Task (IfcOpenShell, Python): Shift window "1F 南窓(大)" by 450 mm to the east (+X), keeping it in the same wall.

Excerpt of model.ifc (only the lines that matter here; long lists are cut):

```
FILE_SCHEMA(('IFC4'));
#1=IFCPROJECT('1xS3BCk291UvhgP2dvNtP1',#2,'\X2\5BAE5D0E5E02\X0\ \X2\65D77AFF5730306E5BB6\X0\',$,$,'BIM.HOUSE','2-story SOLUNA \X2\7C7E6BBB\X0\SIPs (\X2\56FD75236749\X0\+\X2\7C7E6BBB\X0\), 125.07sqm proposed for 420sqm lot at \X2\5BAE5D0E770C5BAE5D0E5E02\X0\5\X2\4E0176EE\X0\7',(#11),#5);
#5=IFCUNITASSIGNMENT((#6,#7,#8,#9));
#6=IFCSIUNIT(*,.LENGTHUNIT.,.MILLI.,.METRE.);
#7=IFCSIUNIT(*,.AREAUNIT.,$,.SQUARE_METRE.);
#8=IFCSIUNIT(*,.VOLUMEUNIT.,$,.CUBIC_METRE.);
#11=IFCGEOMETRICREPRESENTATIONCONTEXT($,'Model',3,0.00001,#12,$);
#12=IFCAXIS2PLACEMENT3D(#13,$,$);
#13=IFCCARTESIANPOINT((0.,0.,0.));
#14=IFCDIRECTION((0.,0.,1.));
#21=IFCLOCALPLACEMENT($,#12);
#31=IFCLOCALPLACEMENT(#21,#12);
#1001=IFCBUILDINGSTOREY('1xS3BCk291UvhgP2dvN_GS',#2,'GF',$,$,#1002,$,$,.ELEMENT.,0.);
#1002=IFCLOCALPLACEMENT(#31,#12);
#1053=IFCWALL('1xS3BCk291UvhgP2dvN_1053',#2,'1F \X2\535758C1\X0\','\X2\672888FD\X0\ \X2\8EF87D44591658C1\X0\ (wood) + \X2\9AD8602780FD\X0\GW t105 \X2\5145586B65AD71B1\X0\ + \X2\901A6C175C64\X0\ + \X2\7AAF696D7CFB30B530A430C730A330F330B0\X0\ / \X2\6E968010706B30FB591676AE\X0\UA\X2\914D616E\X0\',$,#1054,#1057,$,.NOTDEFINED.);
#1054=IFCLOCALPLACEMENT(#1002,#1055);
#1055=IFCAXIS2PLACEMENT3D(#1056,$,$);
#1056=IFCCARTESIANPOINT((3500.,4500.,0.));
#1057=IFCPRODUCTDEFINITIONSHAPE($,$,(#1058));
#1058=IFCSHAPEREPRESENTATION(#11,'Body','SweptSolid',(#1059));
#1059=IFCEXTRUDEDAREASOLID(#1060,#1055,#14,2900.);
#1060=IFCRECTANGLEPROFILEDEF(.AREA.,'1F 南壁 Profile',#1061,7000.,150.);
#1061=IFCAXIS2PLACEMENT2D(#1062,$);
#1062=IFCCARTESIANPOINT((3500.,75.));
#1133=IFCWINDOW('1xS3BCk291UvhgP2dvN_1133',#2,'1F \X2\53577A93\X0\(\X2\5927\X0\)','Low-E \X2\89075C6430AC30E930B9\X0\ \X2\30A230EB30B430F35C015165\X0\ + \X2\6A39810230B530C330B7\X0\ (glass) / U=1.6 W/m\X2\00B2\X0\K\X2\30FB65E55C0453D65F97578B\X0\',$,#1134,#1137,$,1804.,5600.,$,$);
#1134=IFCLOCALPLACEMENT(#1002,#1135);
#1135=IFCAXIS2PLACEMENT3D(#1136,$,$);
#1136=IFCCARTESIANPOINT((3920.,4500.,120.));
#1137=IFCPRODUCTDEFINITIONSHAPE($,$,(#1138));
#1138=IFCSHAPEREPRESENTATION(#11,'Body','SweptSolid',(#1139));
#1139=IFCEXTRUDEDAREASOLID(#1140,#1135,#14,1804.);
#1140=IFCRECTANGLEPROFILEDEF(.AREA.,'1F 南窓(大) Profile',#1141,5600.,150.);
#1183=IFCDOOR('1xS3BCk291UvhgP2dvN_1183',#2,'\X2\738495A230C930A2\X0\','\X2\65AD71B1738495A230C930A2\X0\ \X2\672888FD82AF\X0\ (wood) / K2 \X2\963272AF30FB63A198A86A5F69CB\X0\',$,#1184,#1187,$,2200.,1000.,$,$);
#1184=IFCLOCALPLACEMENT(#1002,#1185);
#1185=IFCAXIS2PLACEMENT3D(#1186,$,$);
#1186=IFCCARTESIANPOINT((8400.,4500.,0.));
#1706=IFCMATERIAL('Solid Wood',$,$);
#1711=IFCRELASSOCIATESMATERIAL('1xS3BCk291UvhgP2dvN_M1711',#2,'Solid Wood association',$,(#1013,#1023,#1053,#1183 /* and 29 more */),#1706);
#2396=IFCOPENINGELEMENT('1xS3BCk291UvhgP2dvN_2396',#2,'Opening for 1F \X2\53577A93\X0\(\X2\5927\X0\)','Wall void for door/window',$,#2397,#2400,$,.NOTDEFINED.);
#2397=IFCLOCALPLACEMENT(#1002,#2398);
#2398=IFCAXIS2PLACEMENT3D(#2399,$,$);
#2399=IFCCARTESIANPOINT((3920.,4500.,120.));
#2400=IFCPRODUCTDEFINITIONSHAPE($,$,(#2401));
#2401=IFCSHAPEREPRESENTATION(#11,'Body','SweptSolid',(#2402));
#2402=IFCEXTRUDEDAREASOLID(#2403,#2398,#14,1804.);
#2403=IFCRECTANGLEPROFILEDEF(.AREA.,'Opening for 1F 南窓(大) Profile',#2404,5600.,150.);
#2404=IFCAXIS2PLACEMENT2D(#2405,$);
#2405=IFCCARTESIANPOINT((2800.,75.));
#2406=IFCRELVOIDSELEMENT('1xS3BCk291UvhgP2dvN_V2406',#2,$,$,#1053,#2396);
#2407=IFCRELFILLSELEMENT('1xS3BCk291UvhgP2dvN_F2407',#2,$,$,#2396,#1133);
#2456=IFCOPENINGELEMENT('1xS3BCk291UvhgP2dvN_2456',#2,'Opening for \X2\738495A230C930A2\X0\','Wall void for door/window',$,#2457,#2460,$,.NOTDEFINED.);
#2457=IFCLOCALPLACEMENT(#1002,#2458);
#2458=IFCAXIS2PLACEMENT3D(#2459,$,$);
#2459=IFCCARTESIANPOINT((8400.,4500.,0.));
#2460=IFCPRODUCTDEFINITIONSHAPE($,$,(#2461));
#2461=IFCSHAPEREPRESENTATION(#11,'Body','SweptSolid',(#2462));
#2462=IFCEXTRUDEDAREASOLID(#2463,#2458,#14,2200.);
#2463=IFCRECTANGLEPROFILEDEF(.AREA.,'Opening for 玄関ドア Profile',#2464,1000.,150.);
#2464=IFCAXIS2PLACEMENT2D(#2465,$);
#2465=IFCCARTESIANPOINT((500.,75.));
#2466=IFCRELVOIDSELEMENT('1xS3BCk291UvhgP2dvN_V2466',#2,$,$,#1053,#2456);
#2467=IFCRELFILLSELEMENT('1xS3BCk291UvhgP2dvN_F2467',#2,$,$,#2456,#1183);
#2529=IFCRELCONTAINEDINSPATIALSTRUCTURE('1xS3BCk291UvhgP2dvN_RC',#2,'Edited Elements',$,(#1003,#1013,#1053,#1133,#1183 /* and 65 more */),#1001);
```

```python
import ifcopenshell
import ifcopenshell.api.geometry
import ifcopenshell.util.placement
import ifcopenshell.util.unit

model = ifcopenshell.open("model.ifc")
unit_scale = ifcopenshell.util.unit.calculate_unit_scale(model)

window = model.by_guid("1xS3BCk291UvhgP2dvN_1133")
opening = window.FillsVoids[0].RelatingOpeningElement
wall = opening.VoidsElements[0].RelatingBuildingElement

wall_matrix = ifcopenshell.util.placement.get_local_placement(wall.ObjectPlacement)
shift = wall_matrix[:3, 0] * 0.45 / unit_scale
before = ifcopenshell.util.placement.get_local_placement(window.ObjectPlacement)[:3, 3].copy()

# The window is not placed relative to its opening, so move both.
for product in (opening, window):
    matrix = ifcopenshell.util.placement.get_local_placement(product.ObjectPlacement)
    matrix[:3, 3] += shift
    ifcopenshell.api.geometry.edit_object_placement(model, product=product, matrix=matrix, is_si=False)

after = ifcopenshell.util.placement.get_local_placement(window.ObjectPlacement)[:3, 3]
print("window moved by", (after - before).round(3) + 0.0)

model.write("model_rev.ifc")
```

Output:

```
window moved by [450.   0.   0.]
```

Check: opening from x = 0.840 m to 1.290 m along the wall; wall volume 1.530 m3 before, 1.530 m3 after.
